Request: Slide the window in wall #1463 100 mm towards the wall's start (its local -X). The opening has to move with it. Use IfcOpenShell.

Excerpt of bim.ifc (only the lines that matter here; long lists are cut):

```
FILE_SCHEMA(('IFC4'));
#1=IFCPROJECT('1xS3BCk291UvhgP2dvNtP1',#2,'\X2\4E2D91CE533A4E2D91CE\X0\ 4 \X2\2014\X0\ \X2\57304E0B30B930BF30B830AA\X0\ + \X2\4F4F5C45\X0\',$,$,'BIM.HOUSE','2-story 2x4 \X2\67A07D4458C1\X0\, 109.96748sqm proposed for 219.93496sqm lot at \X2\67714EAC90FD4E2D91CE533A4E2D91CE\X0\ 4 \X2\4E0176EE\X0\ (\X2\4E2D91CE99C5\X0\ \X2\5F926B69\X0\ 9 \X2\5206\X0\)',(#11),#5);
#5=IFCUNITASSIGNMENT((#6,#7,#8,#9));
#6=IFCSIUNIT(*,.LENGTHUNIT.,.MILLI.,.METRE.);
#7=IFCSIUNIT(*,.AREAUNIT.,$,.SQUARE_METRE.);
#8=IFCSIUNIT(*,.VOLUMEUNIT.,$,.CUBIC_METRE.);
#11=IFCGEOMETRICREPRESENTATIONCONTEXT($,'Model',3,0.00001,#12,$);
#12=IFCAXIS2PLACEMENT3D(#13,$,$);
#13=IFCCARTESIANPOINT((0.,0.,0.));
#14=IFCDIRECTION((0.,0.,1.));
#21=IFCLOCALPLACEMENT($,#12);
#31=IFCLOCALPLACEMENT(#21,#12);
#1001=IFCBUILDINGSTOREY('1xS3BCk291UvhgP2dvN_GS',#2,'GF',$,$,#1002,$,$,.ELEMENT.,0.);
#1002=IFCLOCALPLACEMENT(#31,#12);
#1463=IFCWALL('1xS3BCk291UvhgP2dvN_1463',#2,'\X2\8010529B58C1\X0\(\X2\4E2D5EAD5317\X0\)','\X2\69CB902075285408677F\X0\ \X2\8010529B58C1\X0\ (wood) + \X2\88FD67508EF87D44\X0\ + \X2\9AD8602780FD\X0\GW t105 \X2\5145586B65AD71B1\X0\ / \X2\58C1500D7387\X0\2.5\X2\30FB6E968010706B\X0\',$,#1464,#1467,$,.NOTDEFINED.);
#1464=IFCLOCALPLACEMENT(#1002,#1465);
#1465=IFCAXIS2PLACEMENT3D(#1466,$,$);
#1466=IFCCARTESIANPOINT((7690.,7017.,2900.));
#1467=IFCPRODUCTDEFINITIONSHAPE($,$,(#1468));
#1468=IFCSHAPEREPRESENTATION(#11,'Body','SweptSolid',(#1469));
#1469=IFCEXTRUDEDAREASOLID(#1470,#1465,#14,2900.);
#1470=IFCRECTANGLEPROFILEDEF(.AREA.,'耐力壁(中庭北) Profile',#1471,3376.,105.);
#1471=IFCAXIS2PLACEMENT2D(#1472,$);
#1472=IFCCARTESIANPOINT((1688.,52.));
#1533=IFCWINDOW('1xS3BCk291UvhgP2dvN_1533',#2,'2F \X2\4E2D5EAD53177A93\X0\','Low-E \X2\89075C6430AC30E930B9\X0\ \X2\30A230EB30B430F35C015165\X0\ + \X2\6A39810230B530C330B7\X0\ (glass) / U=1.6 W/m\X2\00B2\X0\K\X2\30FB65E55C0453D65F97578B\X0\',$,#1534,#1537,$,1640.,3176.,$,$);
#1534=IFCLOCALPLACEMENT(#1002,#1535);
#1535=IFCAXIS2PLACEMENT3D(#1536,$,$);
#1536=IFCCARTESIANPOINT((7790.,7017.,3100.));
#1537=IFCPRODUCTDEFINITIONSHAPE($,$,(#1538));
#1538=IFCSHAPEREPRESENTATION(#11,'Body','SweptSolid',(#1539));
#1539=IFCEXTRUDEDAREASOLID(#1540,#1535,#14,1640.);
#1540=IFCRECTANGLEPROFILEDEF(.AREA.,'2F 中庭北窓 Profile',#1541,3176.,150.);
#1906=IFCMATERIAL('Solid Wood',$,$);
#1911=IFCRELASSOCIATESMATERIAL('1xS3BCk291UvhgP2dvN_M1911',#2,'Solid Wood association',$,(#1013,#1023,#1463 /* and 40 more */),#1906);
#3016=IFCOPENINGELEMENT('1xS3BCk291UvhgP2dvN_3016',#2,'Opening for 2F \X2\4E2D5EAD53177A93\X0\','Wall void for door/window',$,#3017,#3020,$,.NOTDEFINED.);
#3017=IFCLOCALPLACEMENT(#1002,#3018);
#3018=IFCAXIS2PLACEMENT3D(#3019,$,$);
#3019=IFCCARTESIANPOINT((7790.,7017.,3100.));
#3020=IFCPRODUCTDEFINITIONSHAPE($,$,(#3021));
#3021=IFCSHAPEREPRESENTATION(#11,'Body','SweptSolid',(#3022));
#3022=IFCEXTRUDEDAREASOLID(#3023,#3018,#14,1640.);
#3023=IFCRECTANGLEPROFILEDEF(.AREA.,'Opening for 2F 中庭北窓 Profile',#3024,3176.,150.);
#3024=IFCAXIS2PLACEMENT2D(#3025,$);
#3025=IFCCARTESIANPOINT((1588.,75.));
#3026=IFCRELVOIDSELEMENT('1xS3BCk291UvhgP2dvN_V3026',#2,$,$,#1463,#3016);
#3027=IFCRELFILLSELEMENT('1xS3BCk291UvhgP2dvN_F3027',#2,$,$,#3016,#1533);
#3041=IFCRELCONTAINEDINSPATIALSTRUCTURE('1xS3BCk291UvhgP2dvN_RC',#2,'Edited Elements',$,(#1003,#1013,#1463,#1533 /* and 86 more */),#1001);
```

```python
import ifcopenshell
import ifcopenshell.api.geometry
import ifcopenshell.util.placement

model = ifcopenshell.open("bim.ifc")

window = model.by_guid("1xS3BCk291UvhgP2dvN_1533")
opening = window.FillsVoids[0].RelatingOpeningElement
wall = opening.VoidsElements[0].RelatingBuildingElement

wall_matrix = ifcopenshell.util.placement.get_local_placement(wall.ObjectPlacement)
shift = wall_matrix[:3, 0] * -100.0
before = ifcopenshell.util.placement.get_local_placement(window.ObjectPlacement)[:3, 3].copy()

# The window is not placed relative to its opening, so move both.
for product in (opening, window):
    matrix = ifcopenshell.util.placement.get_local_placement(product.ObjectPlacement)
    matrix[:3, 3] += shift
    ifcopenshell.api.geometry.edit_object_placement(model, product=product, matrix=matrix, is_si=False)

after = ifcopenshell.util.placement.get_local_placement(window.ObjectPlacement)[:3, 3]
print("window moved by", (after - before).round(3) + 0.0)

model.write("bim_v2.ifc")
```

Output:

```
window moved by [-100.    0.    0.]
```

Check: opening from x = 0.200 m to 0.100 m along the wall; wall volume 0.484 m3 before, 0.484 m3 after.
